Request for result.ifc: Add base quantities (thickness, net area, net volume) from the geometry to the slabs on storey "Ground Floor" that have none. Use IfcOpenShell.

First a look at what the model holds.

```python
import ifcopenshell
import ifcopenshell.util.element
import ifcopenshell.util.unit

model = ifcopenshell.open("result.ifc")
print(model.schema)
for unit_type in ("LENGTHUNIT", "AREAUNIT", "VOLUMEUNIT"):
    print(unit_type, ifcopenshell.util.unit.calculate_unit_scale(model, unit_type))
storey = next(s for s in model.by_type("IfcBuildingStorey") if s.Name == "Ground Floor")
slabs = [e for e in ifcopenshell.util.element.get_decomposition(storey) if e.is_a("IfcSlab")]
for e in sorted(slabs, key=lambda e: e.id()):
    print(e.id(), e.is_a(), e.Name, list(ifcopenshell.util.element.get_psets(e, qtos_only=True)), sep=" | ")
```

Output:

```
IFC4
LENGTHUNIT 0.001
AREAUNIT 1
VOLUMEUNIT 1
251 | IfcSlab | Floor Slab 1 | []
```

```python
import ifcopenshell
import ifcopenshell.api.pset
import ifcopenshell.geom
import ifcopenshell.util.element
import ifcopenshell.util.shape
import ifcopenshell.util.unit

model = ifcopenshell.open("result.ifc")
unit_scale = ifcopenshell.util.unit.calculate_unit_scale(model)
area_scale = ifcopenshell.util.unit.calculate_unit_scale(model, "AREAUNIT")
volume_scale = ifcopenshell.util.unit.calculate_unit_scale(model, "VOLUMEUNIT")
settings = ifcopenshell.geom.settings()

storey = next(s for s in model.by_type("IfcBuildingStorey") if s.Name == "Ground Floor")
slabs = [e for e in ifcopenshell.util.element.get_decomposition(storey) if e.is_a("IfcSlab")]

for e in sorted(slabs, key=lambda e: e.id()):
    if ifcopenshell.util.element.get_psets(e, qtos_only=True, should_inherit=False):
        continue
    # Geometry comes back in metres, in the element's own axes.
    shape = ifcopenshell.geom.create_shape(settings, e)
    values = {
        "Width": ifcopenshell.util.shape.get_z(shape.geometry) / unit_scale,
        "NetArea": ifcopenshell.util.shape.get_footprint_area(shape.geometry) / area_scale,
        "NetVolume": ifcopenshell.util.shape.get_volume(shape.geometry) / volume_scale,
    }
    qto = ifcopenshell.api.pset.add_qto(model, product=e, name="Qto_SlabBaseQuantities")
    ifcopenshell.api.pset.edit_qto(model, qto=qto, properties=values)
    print(e.id(), {k: round(v, 3) for k, v in values.items()})

model.write("result_edited.ifc")
```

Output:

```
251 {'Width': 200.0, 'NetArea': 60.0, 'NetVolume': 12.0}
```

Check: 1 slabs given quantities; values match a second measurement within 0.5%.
